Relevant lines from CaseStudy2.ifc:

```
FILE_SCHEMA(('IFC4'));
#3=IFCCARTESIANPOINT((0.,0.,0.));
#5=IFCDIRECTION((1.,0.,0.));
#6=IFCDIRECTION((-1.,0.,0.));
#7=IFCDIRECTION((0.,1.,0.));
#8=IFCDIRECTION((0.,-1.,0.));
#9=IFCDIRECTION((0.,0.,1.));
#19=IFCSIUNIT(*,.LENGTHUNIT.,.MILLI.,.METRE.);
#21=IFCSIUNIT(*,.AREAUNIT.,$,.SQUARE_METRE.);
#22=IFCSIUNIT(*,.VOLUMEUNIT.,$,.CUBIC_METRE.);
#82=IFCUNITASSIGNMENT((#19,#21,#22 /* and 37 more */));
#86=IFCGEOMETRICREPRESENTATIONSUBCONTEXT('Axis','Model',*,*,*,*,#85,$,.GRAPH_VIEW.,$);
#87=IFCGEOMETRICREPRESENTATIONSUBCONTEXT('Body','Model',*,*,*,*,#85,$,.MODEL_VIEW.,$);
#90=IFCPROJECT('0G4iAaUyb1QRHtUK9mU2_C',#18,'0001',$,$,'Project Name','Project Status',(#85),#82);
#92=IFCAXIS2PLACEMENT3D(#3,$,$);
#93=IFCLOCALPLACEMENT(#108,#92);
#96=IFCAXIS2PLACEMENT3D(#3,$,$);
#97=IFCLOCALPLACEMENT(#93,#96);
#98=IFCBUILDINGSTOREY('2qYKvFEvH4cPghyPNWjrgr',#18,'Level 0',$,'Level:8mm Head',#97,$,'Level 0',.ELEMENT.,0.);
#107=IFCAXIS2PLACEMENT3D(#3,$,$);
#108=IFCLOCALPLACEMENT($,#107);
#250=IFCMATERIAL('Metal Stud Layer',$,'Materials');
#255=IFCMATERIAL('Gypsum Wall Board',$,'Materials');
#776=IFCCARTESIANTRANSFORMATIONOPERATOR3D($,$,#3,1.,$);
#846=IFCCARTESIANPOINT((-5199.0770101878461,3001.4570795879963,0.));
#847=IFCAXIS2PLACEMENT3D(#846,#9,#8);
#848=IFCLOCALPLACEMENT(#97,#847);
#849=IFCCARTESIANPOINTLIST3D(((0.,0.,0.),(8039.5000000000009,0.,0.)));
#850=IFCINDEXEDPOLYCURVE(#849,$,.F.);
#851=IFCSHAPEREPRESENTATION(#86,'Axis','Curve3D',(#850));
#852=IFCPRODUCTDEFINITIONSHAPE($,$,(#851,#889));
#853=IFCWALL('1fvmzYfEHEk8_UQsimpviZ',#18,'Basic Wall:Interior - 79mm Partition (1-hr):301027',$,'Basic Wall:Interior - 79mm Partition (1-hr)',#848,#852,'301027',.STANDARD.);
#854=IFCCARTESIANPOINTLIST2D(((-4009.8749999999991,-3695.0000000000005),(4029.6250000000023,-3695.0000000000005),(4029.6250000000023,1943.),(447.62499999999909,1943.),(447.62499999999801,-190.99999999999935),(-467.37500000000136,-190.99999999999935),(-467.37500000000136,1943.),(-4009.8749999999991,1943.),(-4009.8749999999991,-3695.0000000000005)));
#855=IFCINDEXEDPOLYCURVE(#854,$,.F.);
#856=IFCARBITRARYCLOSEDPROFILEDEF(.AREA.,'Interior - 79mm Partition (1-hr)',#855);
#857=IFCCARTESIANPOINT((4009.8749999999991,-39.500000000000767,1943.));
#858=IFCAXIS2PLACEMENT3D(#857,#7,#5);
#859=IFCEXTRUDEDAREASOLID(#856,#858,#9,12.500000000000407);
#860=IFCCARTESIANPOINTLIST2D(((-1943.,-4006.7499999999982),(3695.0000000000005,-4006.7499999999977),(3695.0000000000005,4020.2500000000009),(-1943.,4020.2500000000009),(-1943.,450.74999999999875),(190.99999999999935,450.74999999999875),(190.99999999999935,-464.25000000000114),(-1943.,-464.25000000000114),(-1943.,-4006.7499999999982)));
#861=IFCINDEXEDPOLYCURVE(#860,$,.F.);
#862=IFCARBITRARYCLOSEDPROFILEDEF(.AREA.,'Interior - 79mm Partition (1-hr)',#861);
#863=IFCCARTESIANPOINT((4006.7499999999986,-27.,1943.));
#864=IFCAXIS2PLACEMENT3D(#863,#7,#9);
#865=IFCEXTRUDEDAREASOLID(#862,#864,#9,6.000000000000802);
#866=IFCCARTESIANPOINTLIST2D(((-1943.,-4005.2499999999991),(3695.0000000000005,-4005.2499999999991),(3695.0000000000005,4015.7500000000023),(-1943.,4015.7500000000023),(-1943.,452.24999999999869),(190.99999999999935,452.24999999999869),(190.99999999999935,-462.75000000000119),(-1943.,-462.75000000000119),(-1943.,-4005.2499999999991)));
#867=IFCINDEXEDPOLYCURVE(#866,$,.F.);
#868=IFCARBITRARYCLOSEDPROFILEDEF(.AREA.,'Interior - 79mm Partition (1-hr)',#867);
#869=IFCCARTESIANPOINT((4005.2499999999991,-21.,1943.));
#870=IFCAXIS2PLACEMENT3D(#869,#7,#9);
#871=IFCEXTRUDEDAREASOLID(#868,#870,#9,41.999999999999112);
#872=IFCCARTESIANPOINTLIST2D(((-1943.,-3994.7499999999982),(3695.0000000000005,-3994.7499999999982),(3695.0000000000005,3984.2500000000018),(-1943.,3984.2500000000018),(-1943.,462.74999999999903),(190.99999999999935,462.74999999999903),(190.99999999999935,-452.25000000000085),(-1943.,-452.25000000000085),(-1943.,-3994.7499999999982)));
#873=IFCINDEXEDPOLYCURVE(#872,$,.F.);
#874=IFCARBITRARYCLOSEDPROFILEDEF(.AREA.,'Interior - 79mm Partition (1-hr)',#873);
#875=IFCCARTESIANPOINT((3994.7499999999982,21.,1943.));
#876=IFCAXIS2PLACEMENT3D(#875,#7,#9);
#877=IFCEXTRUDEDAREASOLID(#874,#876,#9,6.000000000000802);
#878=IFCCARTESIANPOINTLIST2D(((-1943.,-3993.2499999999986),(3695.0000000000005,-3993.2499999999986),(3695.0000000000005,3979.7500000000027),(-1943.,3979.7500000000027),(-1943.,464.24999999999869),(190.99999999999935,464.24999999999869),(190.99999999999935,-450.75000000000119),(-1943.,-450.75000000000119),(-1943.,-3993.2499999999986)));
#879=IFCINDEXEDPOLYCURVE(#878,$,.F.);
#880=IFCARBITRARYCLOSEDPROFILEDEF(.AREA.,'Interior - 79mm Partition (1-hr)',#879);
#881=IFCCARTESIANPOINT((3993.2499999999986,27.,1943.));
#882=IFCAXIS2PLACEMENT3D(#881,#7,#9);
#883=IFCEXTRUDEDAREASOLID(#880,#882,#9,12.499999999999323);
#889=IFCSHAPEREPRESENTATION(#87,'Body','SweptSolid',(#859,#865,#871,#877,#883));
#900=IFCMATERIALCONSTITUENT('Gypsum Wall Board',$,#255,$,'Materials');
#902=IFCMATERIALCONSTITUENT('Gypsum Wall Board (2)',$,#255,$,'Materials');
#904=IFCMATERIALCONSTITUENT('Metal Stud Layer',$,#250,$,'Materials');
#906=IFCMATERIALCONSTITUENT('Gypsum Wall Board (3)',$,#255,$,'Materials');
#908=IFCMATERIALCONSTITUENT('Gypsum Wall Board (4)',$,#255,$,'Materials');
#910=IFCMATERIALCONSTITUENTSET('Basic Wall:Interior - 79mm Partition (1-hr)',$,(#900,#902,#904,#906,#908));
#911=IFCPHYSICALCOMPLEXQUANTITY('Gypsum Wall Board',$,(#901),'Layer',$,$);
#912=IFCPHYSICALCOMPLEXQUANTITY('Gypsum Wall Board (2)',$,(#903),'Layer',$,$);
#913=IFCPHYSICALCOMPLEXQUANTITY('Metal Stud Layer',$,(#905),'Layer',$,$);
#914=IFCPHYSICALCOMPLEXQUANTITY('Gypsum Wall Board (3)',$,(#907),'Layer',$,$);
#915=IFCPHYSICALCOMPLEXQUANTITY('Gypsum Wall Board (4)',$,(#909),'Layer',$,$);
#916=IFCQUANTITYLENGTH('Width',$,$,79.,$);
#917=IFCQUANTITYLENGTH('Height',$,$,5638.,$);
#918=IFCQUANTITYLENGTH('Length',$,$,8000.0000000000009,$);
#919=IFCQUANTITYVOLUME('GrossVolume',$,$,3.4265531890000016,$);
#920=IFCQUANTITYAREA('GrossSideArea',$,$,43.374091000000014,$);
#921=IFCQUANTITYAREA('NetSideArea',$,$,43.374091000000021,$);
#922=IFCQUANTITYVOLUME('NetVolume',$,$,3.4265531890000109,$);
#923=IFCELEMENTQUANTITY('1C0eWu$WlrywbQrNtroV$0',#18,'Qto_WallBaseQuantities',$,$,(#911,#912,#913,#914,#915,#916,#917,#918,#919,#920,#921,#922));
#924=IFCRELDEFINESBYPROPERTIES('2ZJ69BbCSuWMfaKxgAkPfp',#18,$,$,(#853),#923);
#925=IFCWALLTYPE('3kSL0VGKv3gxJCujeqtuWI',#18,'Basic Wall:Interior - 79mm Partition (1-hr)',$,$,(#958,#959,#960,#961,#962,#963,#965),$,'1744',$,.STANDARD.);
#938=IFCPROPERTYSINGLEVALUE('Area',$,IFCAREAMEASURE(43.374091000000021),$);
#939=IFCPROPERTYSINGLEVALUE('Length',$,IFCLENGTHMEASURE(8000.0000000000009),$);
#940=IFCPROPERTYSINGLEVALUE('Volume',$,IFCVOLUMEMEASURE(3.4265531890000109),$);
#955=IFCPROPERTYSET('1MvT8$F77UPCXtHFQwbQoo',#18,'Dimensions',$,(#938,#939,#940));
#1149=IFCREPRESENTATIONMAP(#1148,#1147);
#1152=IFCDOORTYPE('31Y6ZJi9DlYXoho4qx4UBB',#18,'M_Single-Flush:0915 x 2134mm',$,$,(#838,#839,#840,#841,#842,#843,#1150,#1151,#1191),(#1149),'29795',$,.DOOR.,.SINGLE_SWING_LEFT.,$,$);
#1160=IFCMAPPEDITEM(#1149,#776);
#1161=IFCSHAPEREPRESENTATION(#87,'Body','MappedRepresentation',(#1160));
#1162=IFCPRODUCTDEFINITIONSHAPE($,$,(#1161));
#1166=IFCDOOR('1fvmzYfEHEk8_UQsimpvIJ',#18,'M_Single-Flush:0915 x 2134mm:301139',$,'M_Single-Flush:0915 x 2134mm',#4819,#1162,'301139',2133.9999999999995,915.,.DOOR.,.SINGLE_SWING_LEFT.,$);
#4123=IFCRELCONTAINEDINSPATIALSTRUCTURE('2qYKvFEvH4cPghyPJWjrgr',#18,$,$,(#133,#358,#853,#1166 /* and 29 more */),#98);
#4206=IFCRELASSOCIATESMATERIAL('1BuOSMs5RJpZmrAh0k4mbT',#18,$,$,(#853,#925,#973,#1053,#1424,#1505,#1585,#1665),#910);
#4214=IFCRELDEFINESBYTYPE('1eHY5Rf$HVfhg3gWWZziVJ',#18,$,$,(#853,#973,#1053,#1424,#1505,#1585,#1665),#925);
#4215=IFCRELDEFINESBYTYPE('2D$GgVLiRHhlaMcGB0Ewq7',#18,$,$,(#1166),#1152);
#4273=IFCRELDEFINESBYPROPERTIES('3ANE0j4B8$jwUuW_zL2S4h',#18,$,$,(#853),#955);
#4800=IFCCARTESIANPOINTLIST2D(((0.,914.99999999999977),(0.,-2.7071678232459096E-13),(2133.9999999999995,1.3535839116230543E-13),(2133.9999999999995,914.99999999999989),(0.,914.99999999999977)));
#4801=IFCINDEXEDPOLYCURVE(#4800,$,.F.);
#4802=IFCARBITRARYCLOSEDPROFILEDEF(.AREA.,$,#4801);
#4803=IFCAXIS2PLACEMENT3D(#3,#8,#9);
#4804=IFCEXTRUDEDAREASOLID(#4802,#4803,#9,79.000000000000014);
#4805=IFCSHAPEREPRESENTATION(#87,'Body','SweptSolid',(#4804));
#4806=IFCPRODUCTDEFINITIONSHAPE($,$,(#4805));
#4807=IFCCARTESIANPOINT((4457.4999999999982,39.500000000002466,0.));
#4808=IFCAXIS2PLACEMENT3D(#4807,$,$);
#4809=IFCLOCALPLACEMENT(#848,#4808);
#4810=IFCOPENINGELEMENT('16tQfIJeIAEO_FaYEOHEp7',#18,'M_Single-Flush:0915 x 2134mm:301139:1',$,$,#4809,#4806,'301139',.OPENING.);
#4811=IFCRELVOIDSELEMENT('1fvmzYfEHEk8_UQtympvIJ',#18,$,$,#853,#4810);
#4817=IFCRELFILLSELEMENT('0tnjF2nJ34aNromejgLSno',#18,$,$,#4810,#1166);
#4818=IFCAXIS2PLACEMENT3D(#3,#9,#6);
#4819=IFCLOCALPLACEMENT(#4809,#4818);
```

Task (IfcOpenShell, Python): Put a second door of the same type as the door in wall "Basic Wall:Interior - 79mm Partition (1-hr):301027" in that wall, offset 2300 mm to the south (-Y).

```python
import ifcopenshell
import ifcopenshell.api.feature
import ifcopenshell.api.geometry
import ifcopenshell.api.pset
import ifcopenshell.api.root
import ifcopenshell.geom
import ifcopenshell.util.element
import ifcopenshell.util.placement
import ifcopenshell.util.shape
import ifcopenshell.util.unit

model = ifcopenshell.open("CaseStudy2.ifc")
area_scale = ifcopenshell.util.unit.calculate_unit_scale(model, "AREAUNIT")
volume_scale = ifcopenshell.util.unit.calculate_unit_scale(model, "VOLUMEUNIT")
settings = ifcopenshell.geom.settings()


def volume(element):
    """Net volume in cubic metres, openings subtracted."""
    shape = ifcopenshell.geom.create_shape(settings, element)
    return ifcopenshell.util.shape.get_volume(shape.geometry)


def reuse_history(source, copy):
    """copy_class also copies each property set's owner history, people and application; keep the originals."""
    for rel in copy.IsDefinedBy:
        if rel.is_a("IfcRelDefinesByProperties") and (history := rel.RelatingPropertyDefinition.OwnerHistory):
            rel.RelatingPropertyDefinition.OwnerHistory = source.OwnerHistory
            ifcopenshell.util.element.remove_deep2(model, history)


door = model.by_id(1166)
opening = door.FillsVoids[0].RelatingOpeningElement
wall = opening.VoidsElements[0].RelatingBuildingElement
before = volume(wall)
shift = ifcopenshell.util.placement.get_local_placement(wall.ObjectPlacement)[:3, 0] * 2300.0

# copy_class copies the void relationship, type, container and properties, but no geometry.
new_opening = ifcopenshell.api.root.copy_class(model, product=opening)
new_opening.Representation = ifcopenshell.util.element.copy_deep(
    model, opening.Representation, exclude=["IfcGeometricRepresentationContext", "IfcRepresentationMap"]
)
new_opening.Name = "M_Single-Flush:0915 x 2134mm"
new_opening.Tag = None
reuse_history(opening, new_opening)
new_door = ifcopenshell.api.root.copy_class(model, product=door)
new_door.Representation = ifcopenshell.util.element.copy_deep(
    model, door.Representation, exclude=["IfcGeometricRepresentationContext", "IfcRepresentationMap"]
)
new_door.Name = "M_Single-Flush:0915 x 2134mm"
new_door.Tag = None
reuse_history(door, new_door)
ifcopenshell.api.feature.add_filling(model, opening=new_opening, element=new_door)

for old, new in ((opening, new_opening), (door, new_door)):
    matrix = ifcopenshell.util.placement.get_local_placement(old.ObjectPlacement)
    matrix[:3, 3] += shift
    ifcopenshell.api.geometry.edit_object_placement(model, product=new, matrix=matrix, is_si=False)

after = volume(wall)
thickness = 0.079  # wall thickness in metres

# Update the wall's stored quantities.
qto = model.by_id(ifcopenshell.util.element.get_pset(wall, "Qto_WallBaseQuantities", should_inherit=False)["id"])
ifcopenshell.api.pset.edit_qto(model, qto=qto, properties={
    "NetSideArea": after / thickness / area_scale,
    "NetVolume": after / volume_scale,
})
pset = model.by_id(ifcopenshell.util.element.get_pset(wall, "Dimensions", should_inherit=False)["id"])
ifcopenshell.api.pset.edit_pset(model, pset=pset, properties={
    "Area": model.create_entity("IfcAreaMeasure", after / thickness / area_scale),
    "Volume": model.create_entity("IfcVolumeMeasure", after / volume_scale),
})

print(f"wall volume {before:.3f} -> {after:.3f} m3")

model.write("CaseStudy2_rev.ifc")
```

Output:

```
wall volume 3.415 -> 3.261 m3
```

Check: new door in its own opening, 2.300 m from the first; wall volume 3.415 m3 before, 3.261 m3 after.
